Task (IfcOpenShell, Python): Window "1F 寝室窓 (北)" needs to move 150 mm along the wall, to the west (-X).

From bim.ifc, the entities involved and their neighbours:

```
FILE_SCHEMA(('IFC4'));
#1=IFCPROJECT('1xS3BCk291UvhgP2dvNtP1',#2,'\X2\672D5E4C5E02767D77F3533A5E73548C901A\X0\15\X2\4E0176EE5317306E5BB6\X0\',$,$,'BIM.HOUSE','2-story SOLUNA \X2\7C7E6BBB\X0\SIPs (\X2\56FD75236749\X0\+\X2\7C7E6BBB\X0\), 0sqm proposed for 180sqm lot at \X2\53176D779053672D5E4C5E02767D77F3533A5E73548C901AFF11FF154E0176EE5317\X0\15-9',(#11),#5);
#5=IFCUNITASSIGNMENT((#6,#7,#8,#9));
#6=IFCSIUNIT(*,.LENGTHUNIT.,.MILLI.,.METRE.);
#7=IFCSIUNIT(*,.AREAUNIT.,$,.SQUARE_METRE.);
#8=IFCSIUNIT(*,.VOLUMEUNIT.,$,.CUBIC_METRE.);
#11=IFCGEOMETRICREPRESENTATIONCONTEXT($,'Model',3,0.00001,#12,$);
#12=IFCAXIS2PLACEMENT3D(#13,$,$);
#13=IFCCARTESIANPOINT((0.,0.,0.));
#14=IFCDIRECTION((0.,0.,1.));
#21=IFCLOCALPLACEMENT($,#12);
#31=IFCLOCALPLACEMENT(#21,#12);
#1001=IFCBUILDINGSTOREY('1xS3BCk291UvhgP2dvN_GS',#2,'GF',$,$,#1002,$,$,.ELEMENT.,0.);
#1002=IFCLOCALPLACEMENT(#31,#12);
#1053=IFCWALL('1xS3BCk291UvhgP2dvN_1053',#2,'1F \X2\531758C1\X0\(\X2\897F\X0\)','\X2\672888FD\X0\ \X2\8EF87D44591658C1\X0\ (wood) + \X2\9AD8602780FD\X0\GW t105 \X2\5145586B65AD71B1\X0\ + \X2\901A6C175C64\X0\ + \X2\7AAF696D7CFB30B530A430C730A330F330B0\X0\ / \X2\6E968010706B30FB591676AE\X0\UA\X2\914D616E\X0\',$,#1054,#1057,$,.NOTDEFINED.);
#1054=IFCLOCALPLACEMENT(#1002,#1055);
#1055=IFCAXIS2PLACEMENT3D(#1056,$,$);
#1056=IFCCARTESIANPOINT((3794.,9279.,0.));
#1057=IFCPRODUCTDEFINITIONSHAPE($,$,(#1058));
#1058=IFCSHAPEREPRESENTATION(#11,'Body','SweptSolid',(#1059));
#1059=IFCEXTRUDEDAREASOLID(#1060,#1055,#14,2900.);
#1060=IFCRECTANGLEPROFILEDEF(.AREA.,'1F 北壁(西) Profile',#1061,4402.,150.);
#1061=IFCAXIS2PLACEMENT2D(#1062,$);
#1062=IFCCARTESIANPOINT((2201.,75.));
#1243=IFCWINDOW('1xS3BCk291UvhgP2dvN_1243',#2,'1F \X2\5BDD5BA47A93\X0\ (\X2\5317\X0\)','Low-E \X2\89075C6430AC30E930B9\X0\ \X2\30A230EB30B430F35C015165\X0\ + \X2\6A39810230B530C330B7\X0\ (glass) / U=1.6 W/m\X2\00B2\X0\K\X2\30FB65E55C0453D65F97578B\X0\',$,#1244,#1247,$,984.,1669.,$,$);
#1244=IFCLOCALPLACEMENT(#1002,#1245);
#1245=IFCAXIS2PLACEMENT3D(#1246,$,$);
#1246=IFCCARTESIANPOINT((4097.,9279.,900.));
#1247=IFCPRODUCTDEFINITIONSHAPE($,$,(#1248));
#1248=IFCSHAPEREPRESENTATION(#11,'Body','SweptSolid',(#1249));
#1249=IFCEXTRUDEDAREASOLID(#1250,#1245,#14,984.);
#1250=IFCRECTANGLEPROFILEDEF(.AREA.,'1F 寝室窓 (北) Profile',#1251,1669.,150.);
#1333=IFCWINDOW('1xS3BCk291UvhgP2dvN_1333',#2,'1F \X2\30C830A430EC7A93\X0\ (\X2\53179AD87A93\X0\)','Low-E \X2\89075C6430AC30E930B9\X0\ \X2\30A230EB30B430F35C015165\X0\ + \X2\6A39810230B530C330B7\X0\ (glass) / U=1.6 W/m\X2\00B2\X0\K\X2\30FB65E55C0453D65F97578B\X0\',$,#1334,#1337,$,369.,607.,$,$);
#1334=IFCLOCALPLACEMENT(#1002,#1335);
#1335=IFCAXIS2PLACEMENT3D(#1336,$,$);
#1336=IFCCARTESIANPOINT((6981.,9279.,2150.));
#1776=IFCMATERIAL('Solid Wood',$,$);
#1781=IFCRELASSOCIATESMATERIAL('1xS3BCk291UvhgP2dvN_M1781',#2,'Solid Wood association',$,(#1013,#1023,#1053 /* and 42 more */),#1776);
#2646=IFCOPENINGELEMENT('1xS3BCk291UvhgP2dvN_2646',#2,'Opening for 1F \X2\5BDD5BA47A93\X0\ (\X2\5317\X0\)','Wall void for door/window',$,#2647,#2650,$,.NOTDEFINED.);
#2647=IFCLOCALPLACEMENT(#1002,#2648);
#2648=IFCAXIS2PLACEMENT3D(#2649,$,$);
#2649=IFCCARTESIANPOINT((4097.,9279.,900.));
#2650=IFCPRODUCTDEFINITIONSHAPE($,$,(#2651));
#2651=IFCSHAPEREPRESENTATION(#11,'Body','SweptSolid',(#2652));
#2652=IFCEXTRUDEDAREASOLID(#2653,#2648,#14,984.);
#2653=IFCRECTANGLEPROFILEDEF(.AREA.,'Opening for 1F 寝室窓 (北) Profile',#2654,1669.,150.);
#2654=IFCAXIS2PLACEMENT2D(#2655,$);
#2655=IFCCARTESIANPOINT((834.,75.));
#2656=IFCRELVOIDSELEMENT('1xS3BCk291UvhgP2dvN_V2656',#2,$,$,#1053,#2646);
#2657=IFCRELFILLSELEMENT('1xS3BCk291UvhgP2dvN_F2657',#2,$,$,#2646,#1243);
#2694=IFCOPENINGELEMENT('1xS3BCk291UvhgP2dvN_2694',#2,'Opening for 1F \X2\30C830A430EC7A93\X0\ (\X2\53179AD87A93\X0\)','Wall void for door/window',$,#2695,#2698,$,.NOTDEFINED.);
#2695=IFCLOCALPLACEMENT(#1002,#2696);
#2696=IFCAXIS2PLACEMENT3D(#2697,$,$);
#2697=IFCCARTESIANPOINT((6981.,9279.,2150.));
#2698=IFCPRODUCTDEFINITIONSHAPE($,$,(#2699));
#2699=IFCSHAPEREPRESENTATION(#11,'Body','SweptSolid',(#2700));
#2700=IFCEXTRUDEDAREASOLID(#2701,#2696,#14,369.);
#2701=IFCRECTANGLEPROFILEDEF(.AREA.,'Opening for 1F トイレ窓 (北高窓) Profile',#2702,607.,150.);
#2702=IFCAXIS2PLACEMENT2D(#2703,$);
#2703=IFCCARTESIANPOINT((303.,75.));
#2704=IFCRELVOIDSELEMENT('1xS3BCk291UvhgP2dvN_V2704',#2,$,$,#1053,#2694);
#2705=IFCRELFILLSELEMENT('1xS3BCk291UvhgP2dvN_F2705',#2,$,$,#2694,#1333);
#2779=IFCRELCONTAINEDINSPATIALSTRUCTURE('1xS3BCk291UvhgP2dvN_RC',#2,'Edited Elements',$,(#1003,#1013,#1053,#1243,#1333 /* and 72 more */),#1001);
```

```python
import ifcopenshell
import ifcopenshell.api.geometry
import ifcopenshell.util.placement

model = ifcopenshell.open("bim.ifc")

window = model.by_guid("1xS3BCk291UvhgP2dvN_1243")
opening = window.FillsVoids[0].RelatingOpeningElement
wall = opening.VoidsElements[0].RelatingBuildingElement

wall_matrix = ifcopenshell.util.placement.get_local_placement(wall.ObjectPlacement)
shift = wall_matrix[:3, 0] * -150.0
before = ifcopenshell.util.placement.get_local_placement(window.ObjectPlacement)[:3, 3].copy()

# The window is not placed relative to its opening, so move both.
for product in (opening, window):
    matrix = ifcopenshell.util.placement.get_local_placement(product.ObjectPlacement)
    matrix[:3, 3] += shift
    ifcopenshell.api.geometry.edit_object_placement(model, product=product, matrix=matrix, is_si=False)

after = ifcopenshell.util.placement.get_local_placement(window.ObjectPlacement)[:3, 3]
print("window moved by", (after - before).round(3) + 0.0)

model.write("bim_updated.ifc")
```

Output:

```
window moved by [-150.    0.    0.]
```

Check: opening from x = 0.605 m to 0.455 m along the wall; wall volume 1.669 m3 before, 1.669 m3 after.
